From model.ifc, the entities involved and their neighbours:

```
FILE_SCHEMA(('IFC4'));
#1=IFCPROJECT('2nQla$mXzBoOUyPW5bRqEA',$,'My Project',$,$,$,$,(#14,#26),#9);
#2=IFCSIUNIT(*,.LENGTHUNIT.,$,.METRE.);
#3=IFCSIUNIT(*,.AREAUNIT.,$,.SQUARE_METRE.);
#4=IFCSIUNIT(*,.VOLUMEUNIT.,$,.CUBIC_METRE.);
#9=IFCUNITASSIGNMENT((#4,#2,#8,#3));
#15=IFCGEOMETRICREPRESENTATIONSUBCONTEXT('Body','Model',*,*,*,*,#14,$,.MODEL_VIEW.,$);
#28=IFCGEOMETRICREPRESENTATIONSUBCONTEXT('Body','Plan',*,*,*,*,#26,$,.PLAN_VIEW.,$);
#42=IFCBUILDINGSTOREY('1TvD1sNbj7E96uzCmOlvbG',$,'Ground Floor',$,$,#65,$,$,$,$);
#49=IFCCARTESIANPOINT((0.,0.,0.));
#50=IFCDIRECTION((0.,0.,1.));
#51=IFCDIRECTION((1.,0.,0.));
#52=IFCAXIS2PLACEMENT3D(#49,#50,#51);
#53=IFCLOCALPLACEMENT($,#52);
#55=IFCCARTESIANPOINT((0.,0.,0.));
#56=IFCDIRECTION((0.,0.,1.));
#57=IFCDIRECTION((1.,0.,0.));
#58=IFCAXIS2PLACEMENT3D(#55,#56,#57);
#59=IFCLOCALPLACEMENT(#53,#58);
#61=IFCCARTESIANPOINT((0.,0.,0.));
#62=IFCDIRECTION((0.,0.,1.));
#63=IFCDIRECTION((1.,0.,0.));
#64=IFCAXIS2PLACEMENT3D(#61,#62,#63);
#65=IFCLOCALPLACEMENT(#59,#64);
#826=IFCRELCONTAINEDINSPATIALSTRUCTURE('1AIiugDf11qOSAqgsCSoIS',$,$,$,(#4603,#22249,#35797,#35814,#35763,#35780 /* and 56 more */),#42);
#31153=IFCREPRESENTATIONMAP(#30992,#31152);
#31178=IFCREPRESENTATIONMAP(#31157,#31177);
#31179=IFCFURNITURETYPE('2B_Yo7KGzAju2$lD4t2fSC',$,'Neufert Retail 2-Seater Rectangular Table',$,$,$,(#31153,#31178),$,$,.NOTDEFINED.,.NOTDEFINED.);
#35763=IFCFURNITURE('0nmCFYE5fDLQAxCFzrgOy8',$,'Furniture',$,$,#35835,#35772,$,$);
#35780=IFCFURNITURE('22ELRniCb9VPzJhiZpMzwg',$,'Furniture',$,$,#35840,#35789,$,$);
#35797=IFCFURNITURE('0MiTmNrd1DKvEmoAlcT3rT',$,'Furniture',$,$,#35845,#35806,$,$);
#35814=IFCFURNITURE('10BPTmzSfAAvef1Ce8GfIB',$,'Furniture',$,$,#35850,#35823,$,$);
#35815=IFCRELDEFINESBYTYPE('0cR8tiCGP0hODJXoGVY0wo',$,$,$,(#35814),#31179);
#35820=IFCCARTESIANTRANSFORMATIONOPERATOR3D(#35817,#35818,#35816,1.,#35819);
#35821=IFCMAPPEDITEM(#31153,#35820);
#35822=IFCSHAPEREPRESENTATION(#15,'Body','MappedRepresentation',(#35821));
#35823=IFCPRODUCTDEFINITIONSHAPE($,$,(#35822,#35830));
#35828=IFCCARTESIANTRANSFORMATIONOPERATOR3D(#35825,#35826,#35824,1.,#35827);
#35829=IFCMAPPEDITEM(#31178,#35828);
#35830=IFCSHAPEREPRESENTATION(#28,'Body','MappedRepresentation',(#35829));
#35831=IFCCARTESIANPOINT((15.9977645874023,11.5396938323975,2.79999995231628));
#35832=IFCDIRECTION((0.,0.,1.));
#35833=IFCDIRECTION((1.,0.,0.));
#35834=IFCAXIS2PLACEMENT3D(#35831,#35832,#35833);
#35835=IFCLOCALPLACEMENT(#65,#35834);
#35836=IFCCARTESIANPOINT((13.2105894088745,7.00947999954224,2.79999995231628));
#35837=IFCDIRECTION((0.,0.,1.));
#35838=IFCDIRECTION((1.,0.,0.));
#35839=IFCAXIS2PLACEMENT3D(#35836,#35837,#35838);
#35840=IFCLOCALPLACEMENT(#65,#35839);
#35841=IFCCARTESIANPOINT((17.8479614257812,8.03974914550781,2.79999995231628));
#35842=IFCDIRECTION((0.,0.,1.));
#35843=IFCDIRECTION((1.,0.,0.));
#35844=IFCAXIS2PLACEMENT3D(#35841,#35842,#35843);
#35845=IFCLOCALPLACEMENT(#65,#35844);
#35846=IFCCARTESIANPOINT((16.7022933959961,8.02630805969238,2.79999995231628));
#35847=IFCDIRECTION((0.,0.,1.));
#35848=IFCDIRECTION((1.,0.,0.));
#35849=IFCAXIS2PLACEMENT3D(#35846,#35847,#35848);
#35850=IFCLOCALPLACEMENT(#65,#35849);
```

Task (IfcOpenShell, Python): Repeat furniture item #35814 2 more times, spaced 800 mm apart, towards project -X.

```python
import numpy as np
import ifcopenshell
import ifcopenshell.api.geometry
import ifcopenshell.api.root
import ifcopenshell.util.element
import ifcopenshell.util.placement

model = ifcopenshell.open("model.ifc")

source = model.by_guid("10BPTmzSfAAvef1Ce8GfIB")
base = ifcopenshell.util.placement.get_local_placement(source.ObjectPlacement)
step = np.array([-1.0, 0.0, 0.0]) * 0.8

for i in range(1, 3):
    copy = ifcopenshell.api.root.copy_class(model, product=source)
    copy.Representation = ifcopenshell.util.element.copy_deep(
        model, source.Representation, exclude=["IfcGeometricRepresentationContext", "IfcRepresentationMap"]
    )
    matrix = base.copy()
    matrix[:3, 3] += i * step
    print("added at", matrix[:3, 3].round(3) + 0.0)
    ifcopenshell.api.geometry.edit_object_placement(model, product=copy, matrix=matrix, is_si=False)

model.write("model_updated.ifc")
```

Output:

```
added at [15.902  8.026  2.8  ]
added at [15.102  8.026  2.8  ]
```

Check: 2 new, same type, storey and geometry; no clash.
